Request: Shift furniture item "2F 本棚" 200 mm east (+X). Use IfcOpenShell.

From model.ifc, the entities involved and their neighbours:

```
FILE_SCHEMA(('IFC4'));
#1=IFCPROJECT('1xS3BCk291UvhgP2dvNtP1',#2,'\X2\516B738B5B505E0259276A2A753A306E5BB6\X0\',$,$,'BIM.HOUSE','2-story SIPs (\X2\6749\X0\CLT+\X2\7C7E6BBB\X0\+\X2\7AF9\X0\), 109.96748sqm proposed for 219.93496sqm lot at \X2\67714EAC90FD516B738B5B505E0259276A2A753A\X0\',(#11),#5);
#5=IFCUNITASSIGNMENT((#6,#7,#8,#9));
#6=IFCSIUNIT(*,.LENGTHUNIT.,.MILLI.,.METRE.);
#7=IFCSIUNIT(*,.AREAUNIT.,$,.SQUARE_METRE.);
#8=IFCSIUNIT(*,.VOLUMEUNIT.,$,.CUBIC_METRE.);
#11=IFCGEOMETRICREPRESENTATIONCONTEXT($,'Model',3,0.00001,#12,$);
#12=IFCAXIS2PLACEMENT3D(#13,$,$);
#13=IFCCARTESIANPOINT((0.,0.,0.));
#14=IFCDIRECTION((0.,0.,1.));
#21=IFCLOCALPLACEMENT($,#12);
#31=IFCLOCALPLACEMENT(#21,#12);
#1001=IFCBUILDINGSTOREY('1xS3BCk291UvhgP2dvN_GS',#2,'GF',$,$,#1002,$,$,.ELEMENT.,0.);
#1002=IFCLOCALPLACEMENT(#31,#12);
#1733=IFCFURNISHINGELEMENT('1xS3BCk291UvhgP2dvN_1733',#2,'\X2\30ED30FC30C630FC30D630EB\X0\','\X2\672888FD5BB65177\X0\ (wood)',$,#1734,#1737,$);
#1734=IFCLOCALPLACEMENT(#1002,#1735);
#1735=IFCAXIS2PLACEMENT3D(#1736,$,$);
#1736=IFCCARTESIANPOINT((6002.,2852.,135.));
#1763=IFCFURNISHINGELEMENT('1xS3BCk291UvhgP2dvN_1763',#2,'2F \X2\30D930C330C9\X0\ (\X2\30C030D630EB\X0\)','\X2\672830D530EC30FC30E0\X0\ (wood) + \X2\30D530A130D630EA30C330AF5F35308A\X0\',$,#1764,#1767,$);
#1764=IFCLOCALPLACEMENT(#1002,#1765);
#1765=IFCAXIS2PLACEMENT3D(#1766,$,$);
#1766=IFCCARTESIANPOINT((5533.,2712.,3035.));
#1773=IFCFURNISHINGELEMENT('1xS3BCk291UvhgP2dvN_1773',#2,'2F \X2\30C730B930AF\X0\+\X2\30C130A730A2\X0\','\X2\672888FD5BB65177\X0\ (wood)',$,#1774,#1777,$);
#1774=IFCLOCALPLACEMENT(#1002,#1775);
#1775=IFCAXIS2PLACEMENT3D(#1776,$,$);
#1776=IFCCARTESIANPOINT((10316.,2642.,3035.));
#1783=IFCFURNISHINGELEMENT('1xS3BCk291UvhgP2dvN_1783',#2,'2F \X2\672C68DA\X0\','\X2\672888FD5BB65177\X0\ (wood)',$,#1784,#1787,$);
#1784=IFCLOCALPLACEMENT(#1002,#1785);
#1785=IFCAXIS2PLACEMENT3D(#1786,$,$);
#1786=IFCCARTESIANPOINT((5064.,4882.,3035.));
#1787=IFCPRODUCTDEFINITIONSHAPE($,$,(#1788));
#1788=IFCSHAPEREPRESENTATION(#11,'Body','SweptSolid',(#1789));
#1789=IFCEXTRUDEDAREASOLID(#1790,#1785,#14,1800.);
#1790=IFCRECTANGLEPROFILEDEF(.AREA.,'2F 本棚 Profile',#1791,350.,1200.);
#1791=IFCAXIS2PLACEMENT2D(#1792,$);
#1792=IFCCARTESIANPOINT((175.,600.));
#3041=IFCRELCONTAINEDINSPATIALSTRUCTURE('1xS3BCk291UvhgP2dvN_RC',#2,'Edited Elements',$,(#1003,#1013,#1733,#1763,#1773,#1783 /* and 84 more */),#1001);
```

```python
import ifcopenshell
import ifcopenshell.api.geometry
import ifcopenshell.util.placement
import ifcopenshell.util.unit

model = ifcopenshell.open("model.ifc")
unit_scale = ifcopenshell.util.unit.calculate_unit_scale(model)

item = model.by_guid("1xS3BCk291UvhgP2dvN_1783")
matrix = ifcopenshell.util.placement.get_local_placement(item.ObjectPlacement)
matrix[0, 3] += 0.2 / unit_scale
ifcopenshell.api.geometry.edit_object_placement(model, product=item, matrix=matrix, is_si=False)

print(ifcopenshell.util.placement.get_local_placement(item.ObjectPlacement).round(3) + 0.0)

model.write("model_v2.ifc")
```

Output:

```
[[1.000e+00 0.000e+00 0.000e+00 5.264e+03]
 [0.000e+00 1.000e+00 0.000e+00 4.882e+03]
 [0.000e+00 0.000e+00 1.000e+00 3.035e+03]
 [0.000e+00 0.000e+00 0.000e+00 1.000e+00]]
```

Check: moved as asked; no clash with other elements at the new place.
